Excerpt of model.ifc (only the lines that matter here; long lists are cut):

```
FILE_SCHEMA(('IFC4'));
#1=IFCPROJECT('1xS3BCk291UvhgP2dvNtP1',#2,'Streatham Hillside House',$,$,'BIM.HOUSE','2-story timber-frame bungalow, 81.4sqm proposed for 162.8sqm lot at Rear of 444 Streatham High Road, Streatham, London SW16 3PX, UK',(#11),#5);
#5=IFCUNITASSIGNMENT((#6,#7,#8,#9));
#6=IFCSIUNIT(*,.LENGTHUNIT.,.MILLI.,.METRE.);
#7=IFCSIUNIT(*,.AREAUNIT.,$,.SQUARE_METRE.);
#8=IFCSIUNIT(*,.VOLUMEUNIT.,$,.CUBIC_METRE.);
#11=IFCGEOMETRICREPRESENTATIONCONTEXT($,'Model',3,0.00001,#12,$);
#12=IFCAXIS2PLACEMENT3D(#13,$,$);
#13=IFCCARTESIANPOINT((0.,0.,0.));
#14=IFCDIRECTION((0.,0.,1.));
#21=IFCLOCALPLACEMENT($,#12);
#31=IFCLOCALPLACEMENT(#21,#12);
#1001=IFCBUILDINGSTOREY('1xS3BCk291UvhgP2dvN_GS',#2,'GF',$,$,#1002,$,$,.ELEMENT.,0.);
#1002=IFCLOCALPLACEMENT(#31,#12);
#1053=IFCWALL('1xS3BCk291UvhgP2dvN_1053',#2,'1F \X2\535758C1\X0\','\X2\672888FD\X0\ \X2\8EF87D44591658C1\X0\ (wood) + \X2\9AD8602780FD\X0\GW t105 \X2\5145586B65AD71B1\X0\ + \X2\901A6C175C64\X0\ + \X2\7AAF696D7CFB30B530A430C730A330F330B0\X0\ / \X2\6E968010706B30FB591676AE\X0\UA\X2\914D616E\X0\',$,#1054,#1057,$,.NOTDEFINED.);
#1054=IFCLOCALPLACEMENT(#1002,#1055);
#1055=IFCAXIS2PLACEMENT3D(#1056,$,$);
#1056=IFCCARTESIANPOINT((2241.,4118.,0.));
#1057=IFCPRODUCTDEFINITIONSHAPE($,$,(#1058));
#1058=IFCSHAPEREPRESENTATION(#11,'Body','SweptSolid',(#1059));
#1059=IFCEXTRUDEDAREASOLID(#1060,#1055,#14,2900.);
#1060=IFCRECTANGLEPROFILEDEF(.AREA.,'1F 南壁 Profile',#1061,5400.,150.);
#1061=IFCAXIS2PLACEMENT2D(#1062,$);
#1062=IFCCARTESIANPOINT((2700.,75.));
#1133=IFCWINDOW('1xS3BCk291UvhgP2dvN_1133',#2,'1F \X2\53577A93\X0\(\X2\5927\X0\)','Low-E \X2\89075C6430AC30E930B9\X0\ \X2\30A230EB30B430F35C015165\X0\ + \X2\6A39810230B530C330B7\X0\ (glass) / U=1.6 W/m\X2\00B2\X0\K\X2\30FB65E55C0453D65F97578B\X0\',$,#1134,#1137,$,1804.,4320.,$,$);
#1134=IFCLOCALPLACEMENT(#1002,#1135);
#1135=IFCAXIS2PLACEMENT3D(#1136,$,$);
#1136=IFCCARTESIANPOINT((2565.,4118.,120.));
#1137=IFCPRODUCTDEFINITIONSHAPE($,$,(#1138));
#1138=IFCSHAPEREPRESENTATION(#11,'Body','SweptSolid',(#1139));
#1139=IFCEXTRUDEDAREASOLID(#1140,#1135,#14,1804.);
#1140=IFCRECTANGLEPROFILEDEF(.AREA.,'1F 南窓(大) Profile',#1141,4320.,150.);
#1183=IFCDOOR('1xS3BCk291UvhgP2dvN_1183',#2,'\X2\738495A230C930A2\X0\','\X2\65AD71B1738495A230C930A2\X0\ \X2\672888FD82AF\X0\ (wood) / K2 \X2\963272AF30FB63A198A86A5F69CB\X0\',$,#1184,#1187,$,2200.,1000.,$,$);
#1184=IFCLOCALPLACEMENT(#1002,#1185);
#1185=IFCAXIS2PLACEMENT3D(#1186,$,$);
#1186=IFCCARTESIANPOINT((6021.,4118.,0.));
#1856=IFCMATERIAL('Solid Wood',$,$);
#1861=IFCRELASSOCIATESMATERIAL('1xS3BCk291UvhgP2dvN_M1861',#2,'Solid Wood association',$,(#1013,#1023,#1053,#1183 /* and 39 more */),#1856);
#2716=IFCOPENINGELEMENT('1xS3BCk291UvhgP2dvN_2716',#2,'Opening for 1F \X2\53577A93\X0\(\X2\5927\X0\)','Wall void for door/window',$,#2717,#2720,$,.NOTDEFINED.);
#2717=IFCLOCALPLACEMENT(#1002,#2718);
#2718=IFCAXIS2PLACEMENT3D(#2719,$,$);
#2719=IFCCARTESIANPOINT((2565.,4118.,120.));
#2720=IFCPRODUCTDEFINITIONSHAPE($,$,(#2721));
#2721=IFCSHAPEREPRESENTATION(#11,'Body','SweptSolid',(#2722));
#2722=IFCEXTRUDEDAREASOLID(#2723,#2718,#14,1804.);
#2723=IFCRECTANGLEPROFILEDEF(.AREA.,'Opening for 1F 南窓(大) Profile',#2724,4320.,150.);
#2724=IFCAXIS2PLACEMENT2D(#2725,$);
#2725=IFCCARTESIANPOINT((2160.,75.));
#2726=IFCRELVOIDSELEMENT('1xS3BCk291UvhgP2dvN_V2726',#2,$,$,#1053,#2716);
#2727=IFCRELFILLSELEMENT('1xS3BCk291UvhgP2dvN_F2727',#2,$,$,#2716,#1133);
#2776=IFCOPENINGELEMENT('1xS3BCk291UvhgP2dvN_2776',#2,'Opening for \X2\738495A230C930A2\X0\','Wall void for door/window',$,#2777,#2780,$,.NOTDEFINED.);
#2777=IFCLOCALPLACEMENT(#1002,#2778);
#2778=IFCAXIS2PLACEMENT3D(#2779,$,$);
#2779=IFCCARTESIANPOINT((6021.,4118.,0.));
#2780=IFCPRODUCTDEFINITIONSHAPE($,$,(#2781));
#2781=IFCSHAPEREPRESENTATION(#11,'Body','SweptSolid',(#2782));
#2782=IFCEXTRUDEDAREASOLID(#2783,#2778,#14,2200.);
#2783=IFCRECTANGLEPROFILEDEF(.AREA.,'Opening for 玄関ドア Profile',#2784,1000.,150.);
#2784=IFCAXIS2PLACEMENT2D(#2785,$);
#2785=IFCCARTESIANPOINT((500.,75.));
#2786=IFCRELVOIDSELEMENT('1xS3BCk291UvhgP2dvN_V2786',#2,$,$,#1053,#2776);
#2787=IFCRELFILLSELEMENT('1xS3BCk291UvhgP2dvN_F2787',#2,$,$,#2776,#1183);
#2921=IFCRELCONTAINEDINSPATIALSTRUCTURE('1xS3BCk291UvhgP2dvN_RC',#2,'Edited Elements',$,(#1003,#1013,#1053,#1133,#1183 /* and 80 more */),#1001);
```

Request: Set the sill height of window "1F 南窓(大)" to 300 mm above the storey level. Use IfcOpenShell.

```python
import numpy as np
import ifcopenshell
import ifcopenshell.api.geometry
import ifcopenshell.geom
import ifcopenshell.util.element
import ifcopenshell.util.placement
import ifcopenshell.util.shape
import ifcopenshell.util.unit

model = ifcopenshell.open("model.ifc")
unit_scale = ifcopenshell.util.unit.calculate_unit_scale(model)

window = model.by_guid("1xS3BCk291UvhgP2dvN_1133")
opening = window.FillsVoids[0].RelatingOpeningElement
storey = ifcopenshell.util.element.get_container(window, ifc_class="IfcBuildingStorey")
level = ifcopenshell.util.placement.get_local_placement(storey.ObjectPlacement)[2, 3]

# The opening's origin need not be at the sill, so measure its lowest point.
shape = ifcopenshell.geom.create_shape(ifcopenshell.geom.settings(), opening)
bottom = ifcopenshell.util.shape.get_shape_bottom_elevation(shape, shape.geometry) / unit_scale
dz = level + 300.0 - bottom

shift = np.array([0.0, 0.0, dz])
# The window is not placed relative to its opening, so move both.
for product in (opening, window):
    matrix = ifcopenshell.util.placement.get_local_placement(product.ObjectPlacement)
    matrix[:3, 3] += shift
    ifcopenshell.api.geometry.edit_object_placement(model, product=product, matrix=matrix, is_si=False)

print(f"moved by {dz * unit_scale:+.3f} m")

model.write("model_edited.ifc")
```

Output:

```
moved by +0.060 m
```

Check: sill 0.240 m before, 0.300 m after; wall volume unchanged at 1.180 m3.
